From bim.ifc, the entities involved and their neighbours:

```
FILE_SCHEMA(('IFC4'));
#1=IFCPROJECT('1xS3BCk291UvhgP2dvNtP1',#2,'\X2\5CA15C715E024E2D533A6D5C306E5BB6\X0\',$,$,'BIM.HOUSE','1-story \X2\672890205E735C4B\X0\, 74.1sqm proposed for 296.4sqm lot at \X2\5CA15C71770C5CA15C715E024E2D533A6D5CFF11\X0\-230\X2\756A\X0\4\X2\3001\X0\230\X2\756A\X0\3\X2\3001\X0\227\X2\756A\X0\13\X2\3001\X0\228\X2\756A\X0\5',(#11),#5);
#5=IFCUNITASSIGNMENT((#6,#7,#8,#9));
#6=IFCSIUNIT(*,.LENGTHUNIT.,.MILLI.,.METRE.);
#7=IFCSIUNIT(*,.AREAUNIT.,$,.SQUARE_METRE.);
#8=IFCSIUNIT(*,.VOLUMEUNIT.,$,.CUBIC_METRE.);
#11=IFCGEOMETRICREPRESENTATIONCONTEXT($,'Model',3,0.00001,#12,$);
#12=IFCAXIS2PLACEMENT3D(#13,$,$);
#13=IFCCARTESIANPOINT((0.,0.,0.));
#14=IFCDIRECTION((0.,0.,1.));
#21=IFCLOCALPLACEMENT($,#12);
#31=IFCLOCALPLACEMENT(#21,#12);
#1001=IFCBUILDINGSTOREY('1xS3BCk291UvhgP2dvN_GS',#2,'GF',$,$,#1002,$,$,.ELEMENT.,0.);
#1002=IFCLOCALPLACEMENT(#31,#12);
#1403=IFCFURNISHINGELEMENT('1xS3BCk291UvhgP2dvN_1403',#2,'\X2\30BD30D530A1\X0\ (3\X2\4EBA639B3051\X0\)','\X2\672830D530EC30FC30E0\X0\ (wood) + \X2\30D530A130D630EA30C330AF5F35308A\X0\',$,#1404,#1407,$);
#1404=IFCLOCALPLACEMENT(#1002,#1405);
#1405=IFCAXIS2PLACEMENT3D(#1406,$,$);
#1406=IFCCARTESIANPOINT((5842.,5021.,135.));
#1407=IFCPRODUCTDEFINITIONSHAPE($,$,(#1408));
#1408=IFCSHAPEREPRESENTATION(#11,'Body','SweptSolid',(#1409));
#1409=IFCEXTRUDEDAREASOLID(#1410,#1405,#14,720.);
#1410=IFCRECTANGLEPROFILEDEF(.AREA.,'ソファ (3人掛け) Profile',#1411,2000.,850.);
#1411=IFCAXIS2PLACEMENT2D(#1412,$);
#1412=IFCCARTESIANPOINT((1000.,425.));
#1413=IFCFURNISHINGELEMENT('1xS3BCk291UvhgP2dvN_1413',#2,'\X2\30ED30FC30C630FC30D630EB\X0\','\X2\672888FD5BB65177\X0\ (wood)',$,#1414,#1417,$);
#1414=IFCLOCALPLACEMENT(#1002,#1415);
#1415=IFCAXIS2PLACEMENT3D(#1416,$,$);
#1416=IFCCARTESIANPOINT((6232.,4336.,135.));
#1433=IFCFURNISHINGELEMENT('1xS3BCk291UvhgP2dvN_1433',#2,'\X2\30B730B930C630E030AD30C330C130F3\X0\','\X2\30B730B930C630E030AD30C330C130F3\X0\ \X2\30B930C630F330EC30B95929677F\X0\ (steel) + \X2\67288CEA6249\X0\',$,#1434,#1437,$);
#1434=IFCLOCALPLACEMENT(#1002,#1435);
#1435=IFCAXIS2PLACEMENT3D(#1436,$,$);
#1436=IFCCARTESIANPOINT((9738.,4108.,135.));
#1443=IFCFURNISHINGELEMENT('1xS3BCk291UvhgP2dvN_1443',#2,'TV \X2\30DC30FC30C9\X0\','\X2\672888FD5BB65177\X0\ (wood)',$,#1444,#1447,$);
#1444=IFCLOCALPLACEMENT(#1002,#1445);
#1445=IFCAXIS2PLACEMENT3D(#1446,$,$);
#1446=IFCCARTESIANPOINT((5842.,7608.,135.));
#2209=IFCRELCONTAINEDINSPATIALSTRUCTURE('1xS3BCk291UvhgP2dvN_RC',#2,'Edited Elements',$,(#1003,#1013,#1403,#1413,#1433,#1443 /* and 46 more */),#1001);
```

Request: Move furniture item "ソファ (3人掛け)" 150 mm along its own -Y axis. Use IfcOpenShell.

```python
import ifcopenshell
import ifcopenshell.api.geometry
import ifcopenshell.util.placement
import ifcopenshell.util.unit

model = ifcopenshell.open("bim.ifc")
unit_scale = ifcopenshell.util.unit.calculate_unit_scale(model)

item = model.by_id(1403)
matrix = ifcopenshell.util.placement.get_local_placement(item.ObjectPlacement)
matrix[:3, 3] -= matrix[:3, 1] * 0.15 / unit_scale
ifcopenshell.api.geometry.edit_object_placement(model, product=item, matrix=matrix, is_si=False)

print(ifcopenshell.util.placement.get_local_placement(item.ObjectPlacement).round(3) + 0.0)

model.write("bim_edited.ifc")
```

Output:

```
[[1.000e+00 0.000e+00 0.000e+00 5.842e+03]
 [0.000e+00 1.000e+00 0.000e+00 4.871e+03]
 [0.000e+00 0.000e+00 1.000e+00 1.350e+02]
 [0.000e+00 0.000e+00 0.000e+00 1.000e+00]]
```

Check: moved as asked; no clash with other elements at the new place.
